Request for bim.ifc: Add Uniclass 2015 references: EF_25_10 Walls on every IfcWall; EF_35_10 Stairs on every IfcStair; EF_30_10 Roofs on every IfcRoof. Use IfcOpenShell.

First a look at what the model holds.

```python
import ifcopenshell

model = ifcopenshell.open("bim.ifc")
print(model.schema)
print("classifications:", [c.Name for c in model.by_type("IfcClassification")])
for ifc_class in ("IfcDoor", "IfcRoof", "IfcStair", "IfcWall", "IfcWindow"):
    print(ifc_class, len(model.by_type(ifc_class)))
```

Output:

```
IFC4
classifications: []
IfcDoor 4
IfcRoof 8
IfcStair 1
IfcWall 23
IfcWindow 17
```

```python
import ifcopenshell
import ifcopenshell.api.classification

model = ifcopenshell.open("bim.ifc")

system = ifcopenshell.api.classification.add_classification(model, classification="Uniclass 2015")

codes = {
    "IfcWall": ("EF_25_10", "Walls"),
    "IfcStair": ("EF_35_10", "Stairs"),
    "IfcRoof": ("EF_30_10", "Roofs"),
}
for ifc_class, (code, name) in codes.items():
    products = model.by_type(ifc_class)
    ifcopenshell.api.classification.add_reference(
        model, products=products, classification=system, identification=code, name=name
    )
    print(code, len(products))

model.write("bim_v2.ifc")
```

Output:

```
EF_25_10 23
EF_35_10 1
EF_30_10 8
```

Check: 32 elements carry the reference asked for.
